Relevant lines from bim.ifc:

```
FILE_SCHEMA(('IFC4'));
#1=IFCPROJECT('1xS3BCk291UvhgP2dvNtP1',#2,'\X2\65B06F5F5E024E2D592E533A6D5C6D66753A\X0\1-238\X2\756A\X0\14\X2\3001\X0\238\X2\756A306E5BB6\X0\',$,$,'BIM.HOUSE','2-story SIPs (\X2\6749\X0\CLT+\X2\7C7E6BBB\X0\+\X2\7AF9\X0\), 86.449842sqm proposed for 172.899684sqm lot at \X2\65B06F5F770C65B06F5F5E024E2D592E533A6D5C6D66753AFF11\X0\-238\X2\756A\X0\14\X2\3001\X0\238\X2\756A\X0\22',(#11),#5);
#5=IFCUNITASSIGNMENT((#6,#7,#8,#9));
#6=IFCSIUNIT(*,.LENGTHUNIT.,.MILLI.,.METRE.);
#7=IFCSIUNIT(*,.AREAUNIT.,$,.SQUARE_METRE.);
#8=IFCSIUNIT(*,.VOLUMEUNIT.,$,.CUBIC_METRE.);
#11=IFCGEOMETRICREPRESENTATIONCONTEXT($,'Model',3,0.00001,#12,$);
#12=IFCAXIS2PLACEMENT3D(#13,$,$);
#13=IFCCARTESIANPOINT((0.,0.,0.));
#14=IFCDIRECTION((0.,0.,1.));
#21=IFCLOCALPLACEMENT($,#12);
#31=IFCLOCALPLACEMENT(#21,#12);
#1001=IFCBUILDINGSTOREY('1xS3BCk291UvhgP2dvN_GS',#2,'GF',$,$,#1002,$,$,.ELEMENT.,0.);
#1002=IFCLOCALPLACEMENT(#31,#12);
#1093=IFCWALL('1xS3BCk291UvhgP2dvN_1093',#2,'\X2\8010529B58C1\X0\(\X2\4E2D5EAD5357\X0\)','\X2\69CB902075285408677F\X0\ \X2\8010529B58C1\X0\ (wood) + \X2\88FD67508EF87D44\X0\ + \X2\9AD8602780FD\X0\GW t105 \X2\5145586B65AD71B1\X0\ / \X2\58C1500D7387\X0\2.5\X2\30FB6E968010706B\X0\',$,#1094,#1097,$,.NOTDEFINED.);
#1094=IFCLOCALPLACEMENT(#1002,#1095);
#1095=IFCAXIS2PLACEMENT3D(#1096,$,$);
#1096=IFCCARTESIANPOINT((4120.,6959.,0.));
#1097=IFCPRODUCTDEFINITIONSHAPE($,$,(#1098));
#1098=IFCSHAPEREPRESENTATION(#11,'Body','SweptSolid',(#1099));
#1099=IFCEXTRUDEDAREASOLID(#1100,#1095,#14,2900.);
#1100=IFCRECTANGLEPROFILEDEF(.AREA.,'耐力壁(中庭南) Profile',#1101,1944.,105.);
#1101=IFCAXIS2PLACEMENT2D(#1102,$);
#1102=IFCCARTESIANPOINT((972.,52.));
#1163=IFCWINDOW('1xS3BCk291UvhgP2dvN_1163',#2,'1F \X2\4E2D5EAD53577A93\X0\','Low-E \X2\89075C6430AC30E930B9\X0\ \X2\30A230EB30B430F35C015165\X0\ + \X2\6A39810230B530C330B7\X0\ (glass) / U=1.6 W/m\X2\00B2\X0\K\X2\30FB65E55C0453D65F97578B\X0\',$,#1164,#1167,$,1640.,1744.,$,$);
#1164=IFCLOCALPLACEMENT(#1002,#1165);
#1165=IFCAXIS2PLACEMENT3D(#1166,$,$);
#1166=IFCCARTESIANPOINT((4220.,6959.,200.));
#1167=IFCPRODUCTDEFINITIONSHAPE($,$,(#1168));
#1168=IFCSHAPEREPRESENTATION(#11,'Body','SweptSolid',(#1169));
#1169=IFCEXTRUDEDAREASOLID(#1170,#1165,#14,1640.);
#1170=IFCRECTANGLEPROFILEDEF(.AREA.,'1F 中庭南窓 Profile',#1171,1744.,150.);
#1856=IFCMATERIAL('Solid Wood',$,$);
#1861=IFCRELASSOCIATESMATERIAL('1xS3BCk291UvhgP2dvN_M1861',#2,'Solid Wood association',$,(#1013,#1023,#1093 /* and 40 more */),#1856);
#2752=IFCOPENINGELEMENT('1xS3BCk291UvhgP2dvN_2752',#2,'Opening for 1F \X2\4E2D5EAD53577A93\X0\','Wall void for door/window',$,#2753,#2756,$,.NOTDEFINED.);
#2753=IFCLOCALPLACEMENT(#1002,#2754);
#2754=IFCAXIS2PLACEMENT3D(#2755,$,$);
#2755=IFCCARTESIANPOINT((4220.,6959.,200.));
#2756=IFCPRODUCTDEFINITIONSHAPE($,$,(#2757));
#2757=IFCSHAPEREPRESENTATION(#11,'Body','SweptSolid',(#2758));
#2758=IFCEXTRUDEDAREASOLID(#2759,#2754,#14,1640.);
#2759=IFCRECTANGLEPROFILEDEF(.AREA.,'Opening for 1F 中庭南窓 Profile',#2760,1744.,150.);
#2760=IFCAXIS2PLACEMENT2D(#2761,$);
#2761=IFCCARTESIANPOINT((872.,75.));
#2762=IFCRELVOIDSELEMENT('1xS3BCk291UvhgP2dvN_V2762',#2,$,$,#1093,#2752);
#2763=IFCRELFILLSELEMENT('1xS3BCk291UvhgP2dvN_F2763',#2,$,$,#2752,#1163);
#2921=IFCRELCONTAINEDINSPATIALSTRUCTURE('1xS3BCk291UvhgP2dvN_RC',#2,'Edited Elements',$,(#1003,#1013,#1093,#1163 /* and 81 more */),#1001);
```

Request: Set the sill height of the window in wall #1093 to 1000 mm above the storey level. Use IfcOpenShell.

```python
import numpy as np
import ifcopenshell
import ifcopenshell.api.geometry
import ifcopenshell.geom
import ifcopenshell.util.element
import ifcopenshell.util.placement
import ifcopenshell.util.shape
import ifcopenshell.util.unit

model = ifcopenshell.open("bim.ifc")
unit_scale = ifcopenshell.util.unit.calculate_unit_scale(model)

window = model.by_guid("1xS3BCk291UvhgP2dvN_1163")
opening = window.FillsVoids[0].RelatingOpeningElement
storey = ifcopenshell.util.element.get_container(window, ifc_class="IfcBuildingStorey")
level = ifcopenshell.util.placement.get_local_placement(storey.ObjectPlacement)[2, 3]

# The opening's origin need not be at the sill, so measure its lowest point.
shape = ifcopenshell.geom.create_shape(ifcopenshell.geom.settings(), opening)
bottom = ifcopenshell.util.shape.get_shape_bottom_elevation(shape, shape.geometry) / unit_scale
dz = level + 1000.0 - bottom

shift = np.array([0.0, 0.0, dz])
# The window is not placed relative to its opening, so move both.
for product in (opening, window):
    matrix = ifcopenshell.util.placement.get_local_placement(product.ObjectPlacement)
    matrix[:3, 3] += shift
    ifcopenshell.api.geometry.edit_object_placement(model, product=product, matrix=matrix, is_si=False)

print(f"moved by {dz * unit_scale:+.3f} m")

model.write("bim-out.ifc")
```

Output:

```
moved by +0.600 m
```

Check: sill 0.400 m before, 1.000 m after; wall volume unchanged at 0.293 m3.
